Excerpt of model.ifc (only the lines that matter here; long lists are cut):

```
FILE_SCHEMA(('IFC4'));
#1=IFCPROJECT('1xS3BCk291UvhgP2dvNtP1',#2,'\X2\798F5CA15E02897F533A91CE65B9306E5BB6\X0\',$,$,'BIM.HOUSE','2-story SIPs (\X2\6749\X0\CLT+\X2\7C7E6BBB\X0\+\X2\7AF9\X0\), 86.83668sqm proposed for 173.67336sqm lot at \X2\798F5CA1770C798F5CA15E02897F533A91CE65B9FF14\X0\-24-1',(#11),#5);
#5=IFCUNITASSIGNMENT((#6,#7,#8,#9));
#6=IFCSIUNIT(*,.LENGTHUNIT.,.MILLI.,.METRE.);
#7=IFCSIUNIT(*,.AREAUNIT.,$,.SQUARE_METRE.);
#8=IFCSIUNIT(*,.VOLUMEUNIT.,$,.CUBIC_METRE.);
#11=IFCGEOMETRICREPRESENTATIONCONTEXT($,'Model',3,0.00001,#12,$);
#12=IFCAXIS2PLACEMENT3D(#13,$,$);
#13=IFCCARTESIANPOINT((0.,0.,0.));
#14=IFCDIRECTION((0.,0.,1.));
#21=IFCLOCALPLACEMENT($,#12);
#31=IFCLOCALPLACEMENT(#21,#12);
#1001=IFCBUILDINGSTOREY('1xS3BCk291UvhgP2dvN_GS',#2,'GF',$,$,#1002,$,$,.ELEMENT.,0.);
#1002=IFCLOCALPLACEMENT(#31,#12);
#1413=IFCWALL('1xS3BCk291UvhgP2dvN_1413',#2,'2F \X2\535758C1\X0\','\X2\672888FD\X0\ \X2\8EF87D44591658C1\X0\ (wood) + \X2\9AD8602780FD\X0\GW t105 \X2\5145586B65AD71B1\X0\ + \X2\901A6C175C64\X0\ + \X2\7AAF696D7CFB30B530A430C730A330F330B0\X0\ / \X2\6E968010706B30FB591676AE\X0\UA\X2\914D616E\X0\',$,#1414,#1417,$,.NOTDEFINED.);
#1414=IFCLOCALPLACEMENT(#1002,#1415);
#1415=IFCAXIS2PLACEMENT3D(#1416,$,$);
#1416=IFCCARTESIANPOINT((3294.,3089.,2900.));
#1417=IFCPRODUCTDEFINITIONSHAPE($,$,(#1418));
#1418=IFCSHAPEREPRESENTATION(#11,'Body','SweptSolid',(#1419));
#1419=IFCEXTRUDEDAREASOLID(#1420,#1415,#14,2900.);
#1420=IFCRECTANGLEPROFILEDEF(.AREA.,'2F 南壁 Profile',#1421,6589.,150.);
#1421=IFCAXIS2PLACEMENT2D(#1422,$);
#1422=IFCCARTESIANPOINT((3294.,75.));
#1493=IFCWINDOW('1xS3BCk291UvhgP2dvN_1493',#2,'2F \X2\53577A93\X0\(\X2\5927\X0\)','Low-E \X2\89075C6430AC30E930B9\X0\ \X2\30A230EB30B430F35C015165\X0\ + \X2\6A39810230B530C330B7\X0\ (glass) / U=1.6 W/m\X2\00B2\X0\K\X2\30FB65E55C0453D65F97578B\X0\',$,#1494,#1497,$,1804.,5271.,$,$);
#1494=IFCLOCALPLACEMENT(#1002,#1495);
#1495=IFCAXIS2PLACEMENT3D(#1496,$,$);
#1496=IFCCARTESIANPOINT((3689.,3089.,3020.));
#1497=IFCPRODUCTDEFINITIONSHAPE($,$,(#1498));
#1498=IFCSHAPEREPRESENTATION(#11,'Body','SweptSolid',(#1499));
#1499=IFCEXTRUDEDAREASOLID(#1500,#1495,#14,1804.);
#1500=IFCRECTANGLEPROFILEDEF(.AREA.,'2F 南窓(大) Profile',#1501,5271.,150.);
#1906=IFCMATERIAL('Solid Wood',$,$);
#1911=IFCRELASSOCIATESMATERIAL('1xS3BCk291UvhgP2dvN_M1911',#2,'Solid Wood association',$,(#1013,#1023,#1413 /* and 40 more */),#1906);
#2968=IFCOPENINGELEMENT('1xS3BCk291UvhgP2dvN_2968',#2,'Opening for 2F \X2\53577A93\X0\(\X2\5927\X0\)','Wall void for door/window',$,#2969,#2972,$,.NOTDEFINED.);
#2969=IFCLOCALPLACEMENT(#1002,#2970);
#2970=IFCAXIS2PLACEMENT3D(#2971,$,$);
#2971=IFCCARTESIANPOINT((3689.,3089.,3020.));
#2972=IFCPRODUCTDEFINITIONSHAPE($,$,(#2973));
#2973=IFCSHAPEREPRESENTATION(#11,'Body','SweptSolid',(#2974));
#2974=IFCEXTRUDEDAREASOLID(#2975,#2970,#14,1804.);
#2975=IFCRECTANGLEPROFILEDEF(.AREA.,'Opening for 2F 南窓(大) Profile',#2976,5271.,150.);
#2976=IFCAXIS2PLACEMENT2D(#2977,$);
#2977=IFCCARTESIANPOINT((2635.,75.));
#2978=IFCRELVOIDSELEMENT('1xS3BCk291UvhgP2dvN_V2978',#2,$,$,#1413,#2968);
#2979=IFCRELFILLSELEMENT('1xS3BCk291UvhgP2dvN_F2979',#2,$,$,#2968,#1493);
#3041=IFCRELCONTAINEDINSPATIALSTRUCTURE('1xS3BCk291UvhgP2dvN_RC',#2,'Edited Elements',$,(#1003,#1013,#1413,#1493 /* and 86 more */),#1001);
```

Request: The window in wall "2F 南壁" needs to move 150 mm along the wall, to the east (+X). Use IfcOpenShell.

```python
import ifcopenshell
import ifcopenshell.api.geometry
import ifcopenshell.util.placement

model = ifcopenshell.open("model.ifc")

window = model.by_id(1493)
opening = window.FillsVoids[0].RelatingOpeningElement
wall = opening.VoidsElements[0].RelatingBuildingElement

wall_matrix = ifcopenshell.util.placement.get_local_placement(wall.ObjectPlacement)
shift = wall_matrix[:3, 0] * 150.0
before = ifcopenshell.util.placement.get_local_placement(window.ObjectPlacement)[:3, 3].copy()

# The window is not placed relative to its opening, so move both.
for product in (opening, window):
    matrix = ifcopenshell.util.placement.get_local_placement(product.ObjectPlacement)
    matrix[:3, 3] += shift
    ifcopenshell.api.geometry.edit_object_placement(model, product=product, matrix=matrix, is_si=False)

after = ifcopenshell.util.placement.get_local_placement(window.ObjectPlacement)[:3, 3]
print("window moved by", (after - before).round(3) + 0.0)

model.write("model_updated.ifc")
```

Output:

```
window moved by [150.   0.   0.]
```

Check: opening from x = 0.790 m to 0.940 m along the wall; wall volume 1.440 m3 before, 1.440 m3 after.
